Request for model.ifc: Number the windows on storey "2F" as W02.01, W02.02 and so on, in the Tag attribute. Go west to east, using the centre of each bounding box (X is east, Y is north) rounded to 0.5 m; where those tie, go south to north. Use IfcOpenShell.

First a look at what the model holds.

```python
import ifcopenshell
import ifcopenshell.util.element
import ifcopenshell.util.placement

model = ifcopenshell.open("model.ifc")
print(model.schema)
storey = next(s for s in model.by_type("IfcBuildingStorey") if s.Name == "2F")
windows = [e for e in ifcopenshell.util.element.get_decomposition(storey) if e.is_a("IfcWindow")]
for e in sorted(windows, key=lambda e: e.id()):
    origin = ifcopenshell.util.placement.get_local_placement(e.ObjectPlacement)[:3, 3]
    print(e.id(), e.Tag, e.Name, origin.round(2) + 0.0, sep=" | ")
```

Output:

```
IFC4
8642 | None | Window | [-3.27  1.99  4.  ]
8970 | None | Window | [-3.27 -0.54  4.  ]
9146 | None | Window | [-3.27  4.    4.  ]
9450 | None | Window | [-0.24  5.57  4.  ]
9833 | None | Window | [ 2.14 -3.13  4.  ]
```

```python
import ifcopenshell
import ifcopenshell.geom
import ifcopenshell.util.element
import ifcopenshell.util.shape

model = ifcopenshell.open("model.ifc")
settings = ifcopenshell.geom.settings()
settings.set("use-world-coords", True)


def centre(element):
    shape = ifcopenshell.geom.create_shape(settings, element)
    return ifcopenshell.util.shape.get_bbox_centroid(shape.geometry)


storey = next(s for s in model.by_type("IfcBuildingStorey") if s.Name == "2F")
windows = [e for e in ifcopenshell.util.element.get_decomposition(storey) if e.is_a("IfcWindow")]

# Insertion points can sit at a corner or the storey origin, so sort by the geometry (in metres).
centres = {e: centre(e) for e in windows}
windows.sort(key=lambda e: (round(centres[e][0] / 0.5), centres[e][1]))

for i, e in enumerate(windows, start=1):
    number = f"W02.{i:02d}"
    e.Tag = number
    print(e.id(), number)

model.write("model-out.ifc")
```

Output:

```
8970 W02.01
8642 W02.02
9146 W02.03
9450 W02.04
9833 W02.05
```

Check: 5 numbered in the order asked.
